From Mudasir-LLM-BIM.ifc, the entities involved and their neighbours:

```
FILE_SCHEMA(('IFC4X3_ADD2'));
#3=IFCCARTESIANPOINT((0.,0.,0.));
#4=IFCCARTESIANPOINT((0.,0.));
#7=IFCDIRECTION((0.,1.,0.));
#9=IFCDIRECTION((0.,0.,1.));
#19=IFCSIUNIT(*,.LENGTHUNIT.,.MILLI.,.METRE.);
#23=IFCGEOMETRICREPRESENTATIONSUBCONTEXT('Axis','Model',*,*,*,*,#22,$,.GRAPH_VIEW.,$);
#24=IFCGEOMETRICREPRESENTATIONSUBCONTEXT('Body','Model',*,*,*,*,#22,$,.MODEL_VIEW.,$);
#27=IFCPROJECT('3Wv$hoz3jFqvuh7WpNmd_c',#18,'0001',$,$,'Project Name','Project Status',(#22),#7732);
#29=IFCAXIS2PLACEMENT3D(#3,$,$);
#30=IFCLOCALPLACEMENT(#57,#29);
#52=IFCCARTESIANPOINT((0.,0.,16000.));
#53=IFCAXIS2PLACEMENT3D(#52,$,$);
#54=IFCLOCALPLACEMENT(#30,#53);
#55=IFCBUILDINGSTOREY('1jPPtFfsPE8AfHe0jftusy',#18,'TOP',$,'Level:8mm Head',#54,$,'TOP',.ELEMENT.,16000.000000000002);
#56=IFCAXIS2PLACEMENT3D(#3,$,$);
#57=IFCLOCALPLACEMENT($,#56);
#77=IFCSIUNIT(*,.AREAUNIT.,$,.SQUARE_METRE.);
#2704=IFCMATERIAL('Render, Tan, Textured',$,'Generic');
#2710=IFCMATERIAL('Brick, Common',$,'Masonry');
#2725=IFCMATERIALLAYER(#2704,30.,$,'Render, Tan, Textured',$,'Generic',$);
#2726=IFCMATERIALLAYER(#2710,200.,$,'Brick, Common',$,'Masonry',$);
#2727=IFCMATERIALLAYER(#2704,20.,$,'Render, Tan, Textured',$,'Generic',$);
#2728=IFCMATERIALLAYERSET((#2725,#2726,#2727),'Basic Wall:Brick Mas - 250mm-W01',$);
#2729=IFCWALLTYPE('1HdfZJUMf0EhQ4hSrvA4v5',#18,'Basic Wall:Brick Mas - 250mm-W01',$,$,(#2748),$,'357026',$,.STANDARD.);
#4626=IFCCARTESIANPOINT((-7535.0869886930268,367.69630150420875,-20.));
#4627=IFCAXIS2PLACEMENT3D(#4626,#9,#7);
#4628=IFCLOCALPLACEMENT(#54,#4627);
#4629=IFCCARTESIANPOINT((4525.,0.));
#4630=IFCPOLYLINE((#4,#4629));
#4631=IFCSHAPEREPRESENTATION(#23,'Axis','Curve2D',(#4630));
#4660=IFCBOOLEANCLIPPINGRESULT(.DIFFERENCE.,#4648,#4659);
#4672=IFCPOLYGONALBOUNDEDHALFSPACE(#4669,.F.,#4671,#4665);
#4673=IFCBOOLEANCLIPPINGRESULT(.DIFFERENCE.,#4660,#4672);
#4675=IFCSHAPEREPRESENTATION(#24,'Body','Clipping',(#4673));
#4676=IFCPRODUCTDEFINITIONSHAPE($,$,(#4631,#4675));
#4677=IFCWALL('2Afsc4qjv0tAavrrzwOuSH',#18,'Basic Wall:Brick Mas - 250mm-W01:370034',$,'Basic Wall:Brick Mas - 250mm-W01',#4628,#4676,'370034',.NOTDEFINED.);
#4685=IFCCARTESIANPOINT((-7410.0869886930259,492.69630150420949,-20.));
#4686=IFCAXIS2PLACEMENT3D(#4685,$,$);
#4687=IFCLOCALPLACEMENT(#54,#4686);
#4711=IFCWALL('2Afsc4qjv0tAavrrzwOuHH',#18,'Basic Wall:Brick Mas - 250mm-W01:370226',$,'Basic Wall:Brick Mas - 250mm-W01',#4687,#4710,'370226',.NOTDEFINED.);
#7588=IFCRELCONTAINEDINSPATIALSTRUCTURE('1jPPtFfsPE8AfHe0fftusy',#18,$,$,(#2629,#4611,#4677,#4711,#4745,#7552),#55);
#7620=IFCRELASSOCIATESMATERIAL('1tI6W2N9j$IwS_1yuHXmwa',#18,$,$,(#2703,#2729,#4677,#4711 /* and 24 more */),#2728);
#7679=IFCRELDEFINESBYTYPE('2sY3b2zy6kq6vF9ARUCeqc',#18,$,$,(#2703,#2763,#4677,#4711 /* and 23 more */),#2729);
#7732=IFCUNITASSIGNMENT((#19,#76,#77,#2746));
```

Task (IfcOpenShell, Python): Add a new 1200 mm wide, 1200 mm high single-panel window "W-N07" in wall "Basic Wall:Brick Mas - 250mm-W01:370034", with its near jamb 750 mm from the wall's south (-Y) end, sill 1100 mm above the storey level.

```python
import numpy as np
import ifcopenshell
import ifcopenshell.api.feature
import ifcopenshell.api.geometry
import ifcopenshell.api.root
import ifcopenshell.api.spatial
import ifcopenshell.geom
import ifcopenshell.util.element
import ifcopenshell.util.placement
import ifcopenshell.util.representation
import ifcopenshell.util.shape
import ifcopenshell.util.unit

model = ifcopenshell.open("Mudasir-LLM-BIM.ifc")
unit_scale = ifcopenshell.util.unit.calculate_unit_scale(model)
settings = ifcopenshell.geom.settings()


def volume(element):
    """Net volume in cubic metres, openings subtracted."""
    shape = ifcopenshell.geom.create_shape(settings, element)
    return ifcopenshell.util.shape.get_volume(shape.geometry)


wall = model.by_id(4677)
storey = ifcopenshell.util.element.get_container(wall, ifc_class="IfcBuildingStorey")
context = ifcopenshell.util.representation.get_context(model, "Model", "Body", "MODEL_VIEW")
before = volume(wall)

width, height, from_end, sill = 1.2, 1.2, 0.75, 1.1  # metres

# The wall runs along its own X axis, and the end named is its -X end.
wall_shape = ifcopenshell.geom.create_shape(settings, wall)
x, y, z = ifcopenshell.util.shape.get_vertices(wall_shape.geometry).T
start = x.min() + from_end
face, thickness = float(y.min()), float(y.max() - y.min())
wall_matrix = ifcopenshell.util.placement.get_local_placement(wall.ObjectPlacement)
level = ifcopenshell.util.placement.get_local_placement(storey.ObjectPlacement)[2, 3]


def in_wall(x, y):
    """Placement at x, y metres in the wall's axes, at sill height."""
    matrix = wall_matrix.copy()
    matrix[:, 3] = wall_matrix @ np.array([x / unit_scale, y / unit_scale, 0.0, 1.0])
    matrix[2, 3] = level + sill / unit_scale
    return matrix


# Opening: a box that overshoots both wall faces by 50 mm.
opening = ifcopenshell.api.root.create_entity(model, ifc_class="IfcOpeningElement", predefined_type="OPENING")
box = ifcopenshell.api.geometry.add_wall_representation(
    model, context=context, length=width, height=height, thickness=thickness + 0.1
)
ifcopenshell.api.geometry.assign_representation(model, product=opening, representation=box)
ifcopenshell.api.geometry.edit_object_placement(model, product=opening, matrix=in_wall(start, face - 0.05), is_si=False)
ifcopenshell.api.feature.add_feature(model, feature=opening, element=wall)

window = ifcopenshell.api.root.create_entity(model, ifc_class="IfcWindow", name="W-N07", predefined_type="WINDOW")
window.OverallWidth, window.OverallHeight = width / unit_scale, height / unit_scale
window.PartitioningType = "SINGLE_PANEL"
body = ifcopenshell.api.geometry.add_window_representation(
    model,
    context=context,
    overall_width=window.OverallWidth,
    overall_height=window.OverallHeight,
    partition_type="SINGLE_PANEL",
)
ifcopenshell.api.geometry.assign_representation(model, product=window, representation=body)
ifcopenshell.api.spatial.assign_container(model, products=[window], relating_structure=storey)
ifcopenshell.api.feature.add_filling(model, opening=opening, element=window)

# Centre the window in the wall's thickness.
ifcopenshell.api.geometry.edit_object_placement(model, product=window, matrix=in_wall(start, face), is_si=False)
window_shape = ifcopenshell.geom.create_shape(settings, window)
depth = ifcopenshell.util.shape.get_vertices(window_shape.geometry)[:, 1]
offset = face + thickness / 2 - (depth.min() + depth.max()) / 2
ifcopenshell.api.geometry.edit_object_placement(model, product=window, matrix=in_wall(start, offset), is_si=False)

after = volume(wall)

print(f"wall volume {before:.3f} -> {after:.3f} m3")

model.write("Mudasir-LLM-BIM_edited.ifc")
```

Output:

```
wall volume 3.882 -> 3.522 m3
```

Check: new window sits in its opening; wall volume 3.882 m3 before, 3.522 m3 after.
